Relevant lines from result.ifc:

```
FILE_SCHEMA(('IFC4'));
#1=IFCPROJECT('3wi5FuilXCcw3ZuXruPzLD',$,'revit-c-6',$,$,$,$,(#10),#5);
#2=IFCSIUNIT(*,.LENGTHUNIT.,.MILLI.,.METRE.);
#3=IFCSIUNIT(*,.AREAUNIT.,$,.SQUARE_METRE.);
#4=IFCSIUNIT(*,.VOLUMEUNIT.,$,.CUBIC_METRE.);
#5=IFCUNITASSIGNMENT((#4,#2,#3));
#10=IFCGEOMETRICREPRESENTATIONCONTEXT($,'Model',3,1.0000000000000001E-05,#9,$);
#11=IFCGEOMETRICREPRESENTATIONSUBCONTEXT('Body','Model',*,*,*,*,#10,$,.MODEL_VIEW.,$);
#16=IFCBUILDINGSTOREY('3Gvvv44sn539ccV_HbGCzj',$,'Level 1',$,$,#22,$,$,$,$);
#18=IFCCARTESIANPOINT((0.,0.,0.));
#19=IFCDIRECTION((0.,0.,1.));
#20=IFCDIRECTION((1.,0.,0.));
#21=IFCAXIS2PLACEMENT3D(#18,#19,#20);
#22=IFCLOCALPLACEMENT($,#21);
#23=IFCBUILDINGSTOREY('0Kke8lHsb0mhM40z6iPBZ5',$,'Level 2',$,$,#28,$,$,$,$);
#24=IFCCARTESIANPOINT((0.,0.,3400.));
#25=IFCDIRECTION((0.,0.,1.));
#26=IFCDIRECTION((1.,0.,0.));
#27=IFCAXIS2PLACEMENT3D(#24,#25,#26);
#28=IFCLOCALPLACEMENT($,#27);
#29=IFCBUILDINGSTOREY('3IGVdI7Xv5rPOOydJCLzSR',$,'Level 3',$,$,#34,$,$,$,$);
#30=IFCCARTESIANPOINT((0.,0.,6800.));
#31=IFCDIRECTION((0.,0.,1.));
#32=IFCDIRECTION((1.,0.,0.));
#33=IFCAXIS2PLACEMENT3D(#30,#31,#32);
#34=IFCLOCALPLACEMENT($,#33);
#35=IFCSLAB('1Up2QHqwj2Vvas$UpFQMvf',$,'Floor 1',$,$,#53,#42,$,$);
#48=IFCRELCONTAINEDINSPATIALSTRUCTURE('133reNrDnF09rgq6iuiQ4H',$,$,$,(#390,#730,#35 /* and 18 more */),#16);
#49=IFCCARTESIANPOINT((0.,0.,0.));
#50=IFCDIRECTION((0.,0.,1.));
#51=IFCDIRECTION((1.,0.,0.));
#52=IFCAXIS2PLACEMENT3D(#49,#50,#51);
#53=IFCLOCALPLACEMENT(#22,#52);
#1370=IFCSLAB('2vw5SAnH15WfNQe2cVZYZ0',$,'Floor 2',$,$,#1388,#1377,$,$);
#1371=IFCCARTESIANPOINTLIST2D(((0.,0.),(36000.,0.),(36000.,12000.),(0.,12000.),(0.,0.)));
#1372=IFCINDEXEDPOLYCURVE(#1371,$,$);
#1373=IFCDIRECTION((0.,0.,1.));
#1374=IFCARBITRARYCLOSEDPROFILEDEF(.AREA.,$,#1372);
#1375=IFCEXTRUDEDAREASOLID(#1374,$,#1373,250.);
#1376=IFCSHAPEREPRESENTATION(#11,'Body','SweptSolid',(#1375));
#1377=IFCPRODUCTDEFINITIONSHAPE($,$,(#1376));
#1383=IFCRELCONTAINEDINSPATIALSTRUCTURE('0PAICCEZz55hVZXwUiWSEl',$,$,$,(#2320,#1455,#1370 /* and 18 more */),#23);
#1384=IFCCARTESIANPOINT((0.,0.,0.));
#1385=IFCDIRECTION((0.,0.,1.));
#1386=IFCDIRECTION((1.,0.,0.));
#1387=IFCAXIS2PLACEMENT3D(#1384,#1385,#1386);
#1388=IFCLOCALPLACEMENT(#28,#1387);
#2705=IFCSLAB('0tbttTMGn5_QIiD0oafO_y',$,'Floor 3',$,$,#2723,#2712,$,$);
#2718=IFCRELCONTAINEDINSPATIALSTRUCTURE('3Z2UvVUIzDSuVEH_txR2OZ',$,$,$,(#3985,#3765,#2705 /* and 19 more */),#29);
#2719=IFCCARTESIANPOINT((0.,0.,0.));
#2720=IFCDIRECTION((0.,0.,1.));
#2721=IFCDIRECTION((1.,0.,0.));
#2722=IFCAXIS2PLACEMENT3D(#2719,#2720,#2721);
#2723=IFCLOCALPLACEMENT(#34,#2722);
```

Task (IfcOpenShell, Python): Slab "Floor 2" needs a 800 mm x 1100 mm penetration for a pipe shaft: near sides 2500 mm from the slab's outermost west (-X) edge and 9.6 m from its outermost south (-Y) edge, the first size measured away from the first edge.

```python
import numpy as np
import ifcopenshell
import ifcopenshell.api.feature
import ifcopenshell.api.geometry
import ifcopenshell.api.root
import ifcopenshell.geom
import ifcopenshell.util.placement
import ifcopenshell.util.representation
import ifcopenshell.util.shape
import ifcopenshell.util.unit

model = ifcopenshell.open("result.ifc")
unit_scale = ifcopenshell.util.unit.calculate_unit_scale(model)
settings = ifcopenshell.geom.settings()


def volume(element):
    """Net volume in cubic metres, openings subtracted."""
    shape = ifcopenshell.geom.create_shape(settings, element)
    return ifcopenshell.util.shape.get_volume(shape.geometry)


slab = model.by_guid("2vw5SAnH15WfNQe2cVZYZ0")
before = volume(slab)

# Extent in the slab's own axes, in metres. The edges named are its -X and -Y sides.
slab_shape = ifcopenshell.geom.create_shape(settings, slab)
vertices = ifcopenshell.util.shape.get_vertices(slab_shape.geometry)
x_min, y_min, bottom = vertices.min(axis=0)
top = vertices[:, 2].max()

opening = ifcopenshell.api.root.create_entity(model, ifc_class="IfcOpeningElement", name="Pipe shaft opening", predefined_type="OPENING")
context = ifcopenshell.util.representation.get_context(model, "Model", "Body", "MODEL_VIEW")
width, depth = 0.8, 1.1
outline = [(0.0, 0.0), (width, 0.0), (width, depth), (0.0, depth), (0.0, 0.0)]
# Overshoot both faces by 50 mm so the cut is clean.
shape = ifcopenshell.api.geometry.add_slab_representation(
    model, context=context, depth=top - bottom + 0.1, polyline=outline
)
ifcopenshell.api.geometry.assign_representation(model, product=opening, representation=shape)

matrix = ifcopenshell.util.placement.get_local_placement(slab.ObjectPlacement)
matrix[:, 3] = matrix @ np.append(np.array([x_min + 2.5, y_min + 9.6, bottom - 0.05]) / unit_scale, 1.0)
ifcopenshell.api.geometry.edit_object_placement(model, product=opening, matrix=matrix, is_si=False)
ifcopenshell.api.feature.add_feature(model, feature=opening, element=slab)

after = volume(slab)

print(f"slab volume {before:.3f} -> {after:.3f} m3")

model.write("result-out.ifc")
```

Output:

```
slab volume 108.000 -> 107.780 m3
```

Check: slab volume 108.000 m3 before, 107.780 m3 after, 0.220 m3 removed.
